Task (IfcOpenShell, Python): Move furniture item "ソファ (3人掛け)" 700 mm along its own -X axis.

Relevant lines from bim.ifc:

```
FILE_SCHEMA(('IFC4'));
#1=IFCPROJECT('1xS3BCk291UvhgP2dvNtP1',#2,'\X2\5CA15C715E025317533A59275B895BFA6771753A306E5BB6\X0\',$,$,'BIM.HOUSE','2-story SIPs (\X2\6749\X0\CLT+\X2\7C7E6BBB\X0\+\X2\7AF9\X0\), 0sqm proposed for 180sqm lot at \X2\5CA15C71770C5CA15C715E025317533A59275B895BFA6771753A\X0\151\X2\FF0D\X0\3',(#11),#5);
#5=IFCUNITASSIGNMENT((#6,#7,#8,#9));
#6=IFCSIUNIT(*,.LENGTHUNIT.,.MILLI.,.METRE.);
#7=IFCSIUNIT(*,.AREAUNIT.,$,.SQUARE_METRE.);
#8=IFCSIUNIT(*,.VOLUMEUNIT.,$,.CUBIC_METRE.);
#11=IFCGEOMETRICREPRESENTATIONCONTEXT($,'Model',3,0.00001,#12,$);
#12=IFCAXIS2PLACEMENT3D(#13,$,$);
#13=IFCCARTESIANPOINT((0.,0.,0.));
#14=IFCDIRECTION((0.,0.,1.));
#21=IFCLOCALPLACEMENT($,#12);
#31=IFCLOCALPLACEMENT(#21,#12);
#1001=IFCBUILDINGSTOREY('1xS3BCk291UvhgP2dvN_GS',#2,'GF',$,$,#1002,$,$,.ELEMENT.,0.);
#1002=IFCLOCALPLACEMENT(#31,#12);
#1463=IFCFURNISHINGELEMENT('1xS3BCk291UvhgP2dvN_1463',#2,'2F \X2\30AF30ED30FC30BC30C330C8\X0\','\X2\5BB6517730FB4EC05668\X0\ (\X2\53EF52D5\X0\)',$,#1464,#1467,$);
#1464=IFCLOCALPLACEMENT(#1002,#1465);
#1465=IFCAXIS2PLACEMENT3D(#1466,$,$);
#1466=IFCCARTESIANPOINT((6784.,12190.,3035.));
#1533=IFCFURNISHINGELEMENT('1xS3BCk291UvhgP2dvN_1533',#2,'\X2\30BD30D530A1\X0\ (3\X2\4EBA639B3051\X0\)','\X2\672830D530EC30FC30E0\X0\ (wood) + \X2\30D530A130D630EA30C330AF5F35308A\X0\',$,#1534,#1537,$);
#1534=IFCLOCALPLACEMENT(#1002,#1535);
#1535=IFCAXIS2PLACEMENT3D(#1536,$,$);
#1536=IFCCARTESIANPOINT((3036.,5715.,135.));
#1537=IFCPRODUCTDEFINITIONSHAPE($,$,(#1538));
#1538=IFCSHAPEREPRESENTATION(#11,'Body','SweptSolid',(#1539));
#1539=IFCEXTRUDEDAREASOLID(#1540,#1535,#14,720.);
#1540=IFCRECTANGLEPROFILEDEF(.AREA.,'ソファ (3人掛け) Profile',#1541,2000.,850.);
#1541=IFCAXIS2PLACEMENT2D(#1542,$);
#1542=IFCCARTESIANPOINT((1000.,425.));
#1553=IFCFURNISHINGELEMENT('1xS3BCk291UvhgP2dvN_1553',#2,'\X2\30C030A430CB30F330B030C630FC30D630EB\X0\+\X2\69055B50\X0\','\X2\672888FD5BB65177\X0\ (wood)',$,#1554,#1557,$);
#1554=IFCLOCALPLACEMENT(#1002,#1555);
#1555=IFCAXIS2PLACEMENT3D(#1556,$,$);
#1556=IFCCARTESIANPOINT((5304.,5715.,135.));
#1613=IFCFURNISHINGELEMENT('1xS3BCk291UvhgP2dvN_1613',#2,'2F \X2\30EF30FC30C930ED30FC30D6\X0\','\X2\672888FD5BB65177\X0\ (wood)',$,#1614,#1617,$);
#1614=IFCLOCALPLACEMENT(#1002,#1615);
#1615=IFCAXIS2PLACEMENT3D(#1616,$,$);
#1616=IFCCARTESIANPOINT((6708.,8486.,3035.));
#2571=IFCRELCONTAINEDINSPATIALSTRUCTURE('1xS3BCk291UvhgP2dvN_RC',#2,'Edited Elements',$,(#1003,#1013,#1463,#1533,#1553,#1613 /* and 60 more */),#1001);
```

```python
import ifcopenshell
import ifcopenshell.api.geometry
import ifcopenshell.util.placement
import ifcopenshell.util.unit

model = ifcopenshell.open("bim.ifc")
unit_scale = ifcopenshell.util.unit.calculate_unit_scale(model)

item = model.by_guid("1xS3BCk291UvhgP2dvN_1533")
matrix = ifcopenshell.util.placement.get_local_placement(item.ObjectPlacement)
matrix[:3, 3] -= matrix[:3, 0] * 0.7 / unit_scale
ifcopenshell.api.geometry.edit_object_placement(model, product=item, matrix=matrix, is_si=False)

print(ifcopenshell.util.placement.get_local_placement(item.ObjectPlacement).round(3) + 0.0)

model.write("bim_edited.ifc")
```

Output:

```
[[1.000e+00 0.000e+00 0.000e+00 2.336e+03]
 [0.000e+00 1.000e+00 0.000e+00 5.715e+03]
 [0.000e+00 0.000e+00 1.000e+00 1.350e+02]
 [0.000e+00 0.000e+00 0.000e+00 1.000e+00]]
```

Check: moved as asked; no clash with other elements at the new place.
